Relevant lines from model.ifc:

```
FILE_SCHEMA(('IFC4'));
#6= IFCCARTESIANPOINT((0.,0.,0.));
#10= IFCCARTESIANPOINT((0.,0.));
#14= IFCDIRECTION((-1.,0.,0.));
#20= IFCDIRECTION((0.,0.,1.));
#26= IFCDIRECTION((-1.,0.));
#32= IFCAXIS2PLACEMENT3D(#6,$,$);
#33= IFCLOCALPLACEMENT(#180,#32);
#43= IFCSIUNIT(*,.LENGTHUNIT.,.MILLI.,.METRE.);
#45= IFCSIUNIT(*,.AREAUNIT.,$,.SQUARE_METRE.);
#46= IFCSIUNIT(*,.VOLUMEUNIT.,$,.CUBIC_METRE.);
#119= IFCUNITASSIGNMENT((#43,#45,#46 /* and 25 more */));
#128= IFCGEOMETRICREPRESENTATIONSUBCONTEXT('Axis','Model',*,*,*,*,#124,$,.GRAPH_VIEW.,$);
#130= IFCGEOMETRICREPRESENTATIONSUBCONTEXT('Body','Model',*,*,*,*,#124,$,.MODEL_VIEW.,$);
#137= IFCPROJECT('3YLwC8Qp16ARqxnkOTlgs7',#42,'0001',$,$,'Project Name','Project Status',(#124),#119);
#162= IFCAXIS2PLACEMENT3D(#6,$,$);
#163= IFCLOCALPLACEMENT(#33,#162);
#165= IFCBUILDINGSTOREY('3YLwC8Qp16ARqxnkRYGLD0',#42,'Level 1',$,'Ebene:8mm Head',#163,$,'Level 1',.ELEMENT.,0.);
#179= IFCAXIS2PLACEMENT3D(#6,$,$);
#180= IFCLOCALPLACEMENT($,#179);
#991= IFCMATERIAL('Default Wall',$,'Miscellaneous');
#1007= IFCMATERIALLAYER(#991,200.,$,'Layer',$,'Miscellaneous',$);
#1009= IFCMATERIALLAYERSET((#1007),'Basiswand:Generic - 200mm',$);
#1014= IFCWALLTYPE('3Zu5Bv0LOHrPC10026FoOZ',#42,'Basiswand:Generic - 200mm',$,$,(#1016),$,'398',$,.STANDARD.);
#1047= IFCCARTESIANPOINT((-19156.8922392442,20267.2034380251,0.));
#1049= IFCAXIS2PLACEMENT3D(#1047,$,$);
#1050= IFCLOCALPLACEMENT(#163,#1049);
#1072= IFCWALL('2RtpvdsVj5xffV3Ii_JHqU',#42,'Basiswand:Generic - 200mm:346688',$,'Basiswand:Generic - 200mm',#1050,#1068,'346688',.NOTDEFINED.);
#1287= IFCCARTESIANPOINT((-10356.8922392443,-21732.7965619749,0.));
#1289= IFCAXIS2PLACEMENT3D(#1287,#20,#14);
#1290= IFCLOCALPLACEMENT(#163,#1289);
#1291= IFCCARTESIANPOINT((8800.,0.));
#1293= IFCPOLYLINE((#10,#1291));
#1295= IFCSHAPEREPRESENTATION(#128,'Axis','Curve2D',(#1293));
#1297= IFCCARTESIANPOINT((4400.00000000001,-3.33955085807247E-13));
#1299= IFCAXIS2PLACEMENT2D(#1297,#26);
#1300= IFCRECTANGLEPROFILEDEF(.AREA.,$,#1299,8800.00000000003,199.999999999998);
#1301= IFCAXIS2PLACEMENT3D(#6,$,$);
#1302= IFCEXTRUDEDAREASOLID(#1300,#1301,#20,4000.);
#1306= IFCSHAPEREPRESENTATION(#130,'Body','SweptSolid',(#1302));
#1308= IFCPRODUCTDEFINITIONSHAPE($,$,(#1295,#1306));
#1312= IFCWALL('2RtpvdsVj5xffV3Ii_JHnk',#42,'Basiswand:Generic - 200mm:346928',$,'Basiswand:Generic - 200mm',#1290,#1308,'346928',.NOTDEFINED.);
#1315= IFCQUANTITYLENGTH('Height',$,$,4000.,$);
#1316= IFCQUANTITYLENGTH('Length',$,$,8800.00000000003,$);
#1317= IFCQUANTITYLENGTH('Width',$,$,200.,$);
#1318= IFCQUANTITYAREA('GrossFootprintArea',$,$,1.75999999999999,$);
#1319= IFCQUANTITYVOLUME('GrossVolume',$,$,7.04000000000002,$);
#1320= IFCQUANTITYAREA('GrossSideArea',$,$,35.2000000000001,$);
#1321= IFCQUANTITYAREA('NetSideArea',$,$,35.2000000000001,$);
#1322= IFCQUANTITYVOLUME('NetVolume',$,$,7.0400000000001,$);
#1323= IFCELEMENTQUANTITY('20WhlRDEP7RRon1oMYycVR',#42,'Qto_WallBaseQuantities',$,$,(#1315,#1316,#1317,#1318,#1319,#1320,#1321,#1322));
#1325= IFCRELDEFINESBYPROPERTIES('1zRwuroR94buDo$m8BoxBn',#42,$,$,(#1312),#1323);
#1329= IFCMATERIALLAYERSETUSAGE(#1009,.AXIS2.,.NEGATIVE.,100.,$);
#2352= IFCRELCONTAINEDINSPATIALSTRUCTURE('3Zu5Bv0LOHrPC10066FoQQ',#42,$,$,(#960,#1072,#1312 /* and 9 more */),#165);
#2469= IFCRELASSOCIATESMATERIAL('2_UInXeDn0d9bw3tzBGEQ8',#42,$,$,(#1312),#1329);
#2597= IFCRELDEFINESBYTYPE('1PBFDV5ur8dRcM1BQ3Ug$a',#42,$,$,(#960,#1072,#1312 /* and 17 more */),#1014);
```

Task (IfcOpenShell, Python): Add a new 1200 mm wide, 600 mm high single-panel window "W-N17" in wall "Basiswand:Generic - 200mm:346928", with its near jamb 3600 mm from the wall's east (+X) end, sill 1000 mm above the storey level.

```python
import numpy as np
import ifcopenshell
import ifcopenshell.api.feature
import ifcopenshell.api.geometry
import ifcopenshell.api.pset
import ifcopenshell.api.root
import ifcopenshell.api.spatial
import ifcopenshell.geom
import ifcopenshell.util.element
import ifcopenshell.util.placement
import ifcopenshell.util.representation
import ifcopenshell.util.shape
import ifcopenshell.util.unit

model = ifcopenshell.open("model.ifc")
unit_scale = ifcopenshell.util.unit.calculate_unit_scale(model)
area_scale = ifcopenshell.util.unit.calculate_unit_scale(model, "AREAUNIT")
volume_scale = ifcopenshell.util.unit.calculate_unit_scale(model, "VOLUMEUNIT")
settings = ifcopenshell.geom.settings()


def volume(element):
    """Net volume in cubic metres, openings subtracted."""
    shape = ifcopenshell.geom.create_shape(settings, element)
    return ifcopenshell.util.shape.get_volume(shape.geometry)


wall = model.by_guid("2RtpvdsVj5xffV3Ii_JHnk")
storey = ifcopenshell.util.element.get_container(wall, ifc_class="IfcBuildingStorey")
context = ifcopenshell.util.representation.get_context(model, "Model", "Body", "MODEL_VIEW")
before = volume(wall)

width, height, from_end, sill = 1.2, 0.6, 3.6, 1  # metres

# The wall runs along its own X axis, and the end named is its -X end.
wall_shape = ifcopenshell.geom.create_shape(settings, wall)
x, y, z = ifcopenshell.util.shape.get_vertices(wall_shape.geometry).T
start = x.min() + from_end
face, thickness = float(y.min()), float(y.max() - y.min())
wall_matrix = ifcopenshell.util.placement.get_local_placement(wall.ObjectPlacement)
level = ifcopenshell.util.placement.get_local_placement(storey.ObjectPlacement)[2, 3]


def in_wall(x, y):
    """Placement at x, y metres in the wall's axes, at sill height."""
    matrix = wall_matrix.copy()
    matrix[:, 3] = wall_matrix @ np.array([x / unit_scale, y / unit_scale, 0.0, 1.0])
    matrix[2, 3] = level + sill / unit_scale
    return matrix


# Opening: a box that overshoots both wall faces by 50 mm.
opening = ifcopenshell.api.root.create_entity(model, ifc_class="IfcOpeningElement", predefined_type="OPENING")
box = ifcopenshell.api.geometry.add_wall_representation(
    model, context=context, length=width, height=height, thickness=thickness + 0.1
)
ifcopenshell.api.geometry.assign_representation(model, product=opening, representation=box)
ifcopenshell.api.geometry.edit_object_placement(model, product=opening, matrix=in_wall(start, face - 0.05), is_si=False)
ifcopenshell.api.feature.add_feature(model, feature=opening, element=wall)

window = ifcopenshell.api.root.create_entity(model, ifc_class="IfcWindow", name="W-N17", predefined_type="WINDOW")
window.OverallWidth, window.OverallHeight = width / unit_scale, height / unit_scale
window.PartitioningType = "SINGLE_PANEL"
body = ifcopenshell.api.geometry.add_window_representation(
    model,
    context=context,
    overall_width=window.OverallWidth,
    overall_height=window.OverallHeight,
    partition_type="SINGLE_PANEL",
)
ifcopenshell.api.geometry.assign_representation(model, product=window, representation=body)
ifcopenshell.api.spatial.assign_container(model, products=[window], relating_structure=storey)
ifcopenshell.api.feature.add_filling(model, opening=opening, element=window)

# Centre the window in the wall's thickness.
ifcopenshell.api.geometry.edit_object_placement(model, product=window, matrix=in_wall(start, face), is_si=False)
window_shape = ifcopenshell.geom.create_shape(settings, window)
depth = ifcopenshell.util.shape.get_vertices(window_shape.geometry)[:, 1]
offset = face + thickness / 2 - (depth.min() + depth.max()) / 2
ifcopenshell.api.geometry.edit_object_placement(model, product=window, matrix=in_wall(start, offset), is_si=False)

after = volume(wall)

# Update the wall's stored quantities.
qto = model.by_id(ifcopenshell.util.element.get_pset(wall, "Qto_WallBaseQuantities", should_inherit=False)["id"])
ifcopenshell.api.pset.edit_qto(model, qto=qto, properties={
    "NetSideArea": after / thickness / area_scale,
    "NetVolume": after / volume_scale,
})

print(f"wall volume {before:.3f} -> {after:.3f} m3")

model.write("model-out.ifc")
```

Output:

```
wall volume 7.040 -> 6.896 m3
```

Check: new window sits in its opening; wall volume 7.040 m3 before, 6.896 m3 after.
